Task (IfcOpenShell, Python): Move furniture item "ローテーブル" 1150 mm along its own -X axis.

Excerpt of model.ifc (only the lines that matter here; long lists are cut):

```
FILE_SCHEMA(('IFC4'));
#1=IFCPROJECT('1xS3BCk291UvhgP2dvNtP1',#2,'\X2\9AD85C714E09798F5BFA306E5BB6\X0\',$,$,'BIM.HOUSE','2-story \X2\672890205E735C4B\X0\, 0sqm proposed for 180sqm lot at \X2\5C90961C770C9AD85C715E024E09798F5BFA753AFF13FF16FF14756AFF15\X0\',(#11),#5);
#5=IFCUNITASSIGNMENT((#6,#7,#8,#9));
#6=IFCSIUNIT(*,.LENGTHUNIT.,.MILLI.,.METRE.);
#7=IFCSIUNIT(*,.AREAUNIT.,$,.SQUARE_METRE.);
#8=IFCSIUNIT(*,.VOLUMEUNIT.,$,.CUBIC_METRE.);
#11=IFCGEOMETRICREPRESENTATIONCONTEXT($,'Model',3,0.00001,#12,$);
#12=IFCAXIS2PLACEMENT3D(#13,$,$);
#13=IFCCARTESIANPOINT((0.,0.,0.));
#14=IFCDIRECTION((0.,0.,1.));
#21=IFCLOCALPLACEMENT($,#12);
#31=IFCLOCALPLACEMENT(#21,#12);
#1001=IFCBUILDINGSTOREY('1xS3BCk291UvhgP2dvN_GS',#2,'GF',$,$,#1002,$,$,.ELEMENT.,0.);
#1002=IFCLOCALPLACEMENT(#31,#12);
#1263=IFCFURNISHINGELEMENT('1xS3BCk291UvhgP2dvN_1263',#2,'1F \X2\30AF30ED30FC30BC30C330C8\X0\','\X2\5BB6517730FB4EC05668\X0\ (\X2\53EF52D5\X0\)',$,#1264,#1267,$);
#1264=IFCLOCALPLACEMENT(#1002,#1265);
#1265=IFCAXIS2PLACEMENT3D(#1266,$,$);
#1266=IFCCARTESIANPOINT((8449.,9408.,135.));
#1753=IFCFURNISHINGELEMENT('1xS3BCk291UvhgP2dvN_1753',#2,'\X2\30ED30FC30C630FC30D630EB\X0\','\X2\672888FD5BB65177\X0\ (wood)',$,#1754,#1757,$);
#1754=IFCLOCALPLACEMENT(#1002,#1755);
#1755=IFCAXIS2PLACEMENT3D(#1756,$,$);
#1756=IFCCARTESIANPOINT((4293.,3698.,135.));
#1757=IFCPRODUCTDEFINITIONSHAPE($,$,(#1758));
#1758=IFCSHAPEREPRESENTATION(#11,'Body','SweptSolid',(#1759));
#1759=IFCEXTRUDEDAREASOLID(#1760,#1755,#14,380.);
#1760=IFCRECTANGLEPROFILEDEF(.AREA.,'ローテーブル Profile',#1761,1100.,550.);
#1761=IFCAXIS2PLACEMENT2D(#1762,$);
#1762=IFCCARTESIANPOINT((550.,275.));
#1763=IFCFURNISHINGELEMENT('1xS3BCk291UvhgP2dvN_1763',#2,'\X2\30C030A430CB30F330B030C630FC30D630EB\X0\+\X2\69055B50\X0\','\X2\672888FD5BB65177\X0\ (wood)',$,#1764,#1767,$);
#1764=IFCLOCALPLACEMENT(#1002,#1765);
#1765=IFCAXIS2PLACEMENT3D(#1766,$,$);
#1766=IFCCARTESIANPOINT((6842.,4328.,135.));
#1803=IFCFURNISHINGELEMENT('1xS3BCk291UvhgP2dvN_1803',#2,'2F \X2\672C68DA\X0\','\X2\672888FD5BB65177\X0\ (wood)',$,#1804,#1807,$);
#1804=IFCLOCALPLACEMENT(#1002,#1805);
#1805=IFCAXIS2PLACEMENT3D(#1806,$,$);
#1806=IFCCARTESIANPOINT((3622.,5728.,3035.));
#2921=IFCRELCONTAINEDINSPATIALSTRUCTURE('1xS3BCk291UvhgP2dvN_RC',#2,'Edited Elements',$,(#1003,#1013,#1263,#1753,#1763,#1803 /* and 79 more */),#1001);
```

```python
import ifcopenshell
import ifcopenshell.api.geometry
import ifcopenshell.util.placement

model = ifcopenshell.open("model.ifc")

item = model.by_id(1753)
matrix = ifcopenshell.util.placement.get_local_placement(item.ObjectPlacement)
matrix[:3, 3] -= matrix[:3, 0] * 1150.0
ifcopenshell.api.geometry.edit_object_placement(model, product=item, matrix=matrix, is_si=False)

print(ifcopenshell.util.placement.get_local_placement(item.ObjectPlacement).round(3) + 0.0)

model.write("model_edited.ifc")
```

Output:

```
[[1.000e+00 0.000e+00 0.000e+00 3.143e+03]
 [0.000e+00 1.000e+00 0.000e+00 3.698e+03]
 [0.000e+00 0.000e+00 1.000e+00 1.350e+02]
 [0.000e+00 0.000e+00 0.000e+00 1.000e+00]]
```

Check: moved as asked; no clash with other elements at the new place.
